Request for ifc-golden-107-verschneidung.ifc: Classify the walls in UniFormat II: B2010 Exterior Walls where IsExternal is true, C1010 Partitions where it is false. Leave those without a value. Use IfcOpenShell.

First a look at what the model holds.

```python
import ifcopenshell
import ifcopenshell.util.element

model = ifcopenshell.open("ifc-golden-107-verschneidung.ifc")
print(model.schema)
print("classifications:", [c.Name for c in model.by_type("IfcClassification")])
values = [ifcopenshell.util.element.get_pset(e, "Pset_WallCommon", "IsExternal") for e in model.by_type("IfcWall")]
for value in (True, False, None):
    print("IsExternal", value, values.count(value))
```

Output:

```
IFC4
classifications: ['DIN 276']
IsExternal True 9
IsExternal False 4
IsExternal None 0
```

```python
import ifcopenshell
import ifcopenshell.api.classification
import ifcopenshell.util.element

model = ifcopenshell.open("ifc-golden-107-verschneidung.ifc")

system = ifcopenshell.api.classification.add_classification(model, classification="UniFormat II")

walls = model.by_type("IfcWall")
external = {e: ifcopenshell.util.element.get_pset(e, "Pset_WallCommon", "IsExternal") for e in walls}
for flag, code, name in ((True, "B2010", "Exterior Walls"), (False, "C1010", "Partitions")):
    products = [e for e in walls if external[e] is flag]
    ifcopenshell.api.classification.add_reference(
        model, products=products, classification=system, identification=code, name=name
    )
    print(code, len(products))

model.write("ifc-golden-107-verschneidung-out.ifc")
```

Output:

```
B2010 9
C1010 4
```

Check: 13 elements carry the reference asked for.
